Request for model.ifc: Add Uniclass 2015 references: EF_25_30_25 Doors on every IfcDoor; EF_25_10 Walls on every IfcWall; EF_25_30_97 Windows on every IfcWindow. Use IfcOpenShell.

First a look at what the model holds.

```python
import ifcopenshell

model = ifcopenshell.open("model.ifc")
print(model.schema)
print("classifications:", [c.Name for c in model.by_type("IfcClassification")])
for ifc_class in ("IfcDoor", "IfcRoof", "IfcStair", "IfcWall", "IfcWindow"):
    print(ifc_class, len(model.by_type(ifc_class)))
```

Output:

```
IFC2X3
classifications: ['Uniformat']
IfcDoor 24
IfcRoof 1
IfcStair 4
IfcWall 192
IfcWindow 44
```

```python
import ifcopenshell
import ifcopenshell.api.classification

model = ifcopenshell.open("model.ifc")

# IFC2X3 requires Source and Edition and has no link from the project to the system.
system = model.create_entity("IfcClassification", Source="NBS", Edition="2015", Name="Uniclass 2015")

codes = {
    "IfcDoor": ("EF_25_30_25", "Doors"),
    "IfcWall": ("EF_25_10", "Walls"),
    "IfcWindow": ("EF_25_30_97", "Windows"),
}
for ifc_class, (code, name) in codes.items():
    products = model.by_type(ifc_class)
    ifcopenshell.api.classification.add_reference(
        model, products=products, classification=system, identification=code, name=name
    )
    print(code, len(products))

model.write("model_updated.ifc")
```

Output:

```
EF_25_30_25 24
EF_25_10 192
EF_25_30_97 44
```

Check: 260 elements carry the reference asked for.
